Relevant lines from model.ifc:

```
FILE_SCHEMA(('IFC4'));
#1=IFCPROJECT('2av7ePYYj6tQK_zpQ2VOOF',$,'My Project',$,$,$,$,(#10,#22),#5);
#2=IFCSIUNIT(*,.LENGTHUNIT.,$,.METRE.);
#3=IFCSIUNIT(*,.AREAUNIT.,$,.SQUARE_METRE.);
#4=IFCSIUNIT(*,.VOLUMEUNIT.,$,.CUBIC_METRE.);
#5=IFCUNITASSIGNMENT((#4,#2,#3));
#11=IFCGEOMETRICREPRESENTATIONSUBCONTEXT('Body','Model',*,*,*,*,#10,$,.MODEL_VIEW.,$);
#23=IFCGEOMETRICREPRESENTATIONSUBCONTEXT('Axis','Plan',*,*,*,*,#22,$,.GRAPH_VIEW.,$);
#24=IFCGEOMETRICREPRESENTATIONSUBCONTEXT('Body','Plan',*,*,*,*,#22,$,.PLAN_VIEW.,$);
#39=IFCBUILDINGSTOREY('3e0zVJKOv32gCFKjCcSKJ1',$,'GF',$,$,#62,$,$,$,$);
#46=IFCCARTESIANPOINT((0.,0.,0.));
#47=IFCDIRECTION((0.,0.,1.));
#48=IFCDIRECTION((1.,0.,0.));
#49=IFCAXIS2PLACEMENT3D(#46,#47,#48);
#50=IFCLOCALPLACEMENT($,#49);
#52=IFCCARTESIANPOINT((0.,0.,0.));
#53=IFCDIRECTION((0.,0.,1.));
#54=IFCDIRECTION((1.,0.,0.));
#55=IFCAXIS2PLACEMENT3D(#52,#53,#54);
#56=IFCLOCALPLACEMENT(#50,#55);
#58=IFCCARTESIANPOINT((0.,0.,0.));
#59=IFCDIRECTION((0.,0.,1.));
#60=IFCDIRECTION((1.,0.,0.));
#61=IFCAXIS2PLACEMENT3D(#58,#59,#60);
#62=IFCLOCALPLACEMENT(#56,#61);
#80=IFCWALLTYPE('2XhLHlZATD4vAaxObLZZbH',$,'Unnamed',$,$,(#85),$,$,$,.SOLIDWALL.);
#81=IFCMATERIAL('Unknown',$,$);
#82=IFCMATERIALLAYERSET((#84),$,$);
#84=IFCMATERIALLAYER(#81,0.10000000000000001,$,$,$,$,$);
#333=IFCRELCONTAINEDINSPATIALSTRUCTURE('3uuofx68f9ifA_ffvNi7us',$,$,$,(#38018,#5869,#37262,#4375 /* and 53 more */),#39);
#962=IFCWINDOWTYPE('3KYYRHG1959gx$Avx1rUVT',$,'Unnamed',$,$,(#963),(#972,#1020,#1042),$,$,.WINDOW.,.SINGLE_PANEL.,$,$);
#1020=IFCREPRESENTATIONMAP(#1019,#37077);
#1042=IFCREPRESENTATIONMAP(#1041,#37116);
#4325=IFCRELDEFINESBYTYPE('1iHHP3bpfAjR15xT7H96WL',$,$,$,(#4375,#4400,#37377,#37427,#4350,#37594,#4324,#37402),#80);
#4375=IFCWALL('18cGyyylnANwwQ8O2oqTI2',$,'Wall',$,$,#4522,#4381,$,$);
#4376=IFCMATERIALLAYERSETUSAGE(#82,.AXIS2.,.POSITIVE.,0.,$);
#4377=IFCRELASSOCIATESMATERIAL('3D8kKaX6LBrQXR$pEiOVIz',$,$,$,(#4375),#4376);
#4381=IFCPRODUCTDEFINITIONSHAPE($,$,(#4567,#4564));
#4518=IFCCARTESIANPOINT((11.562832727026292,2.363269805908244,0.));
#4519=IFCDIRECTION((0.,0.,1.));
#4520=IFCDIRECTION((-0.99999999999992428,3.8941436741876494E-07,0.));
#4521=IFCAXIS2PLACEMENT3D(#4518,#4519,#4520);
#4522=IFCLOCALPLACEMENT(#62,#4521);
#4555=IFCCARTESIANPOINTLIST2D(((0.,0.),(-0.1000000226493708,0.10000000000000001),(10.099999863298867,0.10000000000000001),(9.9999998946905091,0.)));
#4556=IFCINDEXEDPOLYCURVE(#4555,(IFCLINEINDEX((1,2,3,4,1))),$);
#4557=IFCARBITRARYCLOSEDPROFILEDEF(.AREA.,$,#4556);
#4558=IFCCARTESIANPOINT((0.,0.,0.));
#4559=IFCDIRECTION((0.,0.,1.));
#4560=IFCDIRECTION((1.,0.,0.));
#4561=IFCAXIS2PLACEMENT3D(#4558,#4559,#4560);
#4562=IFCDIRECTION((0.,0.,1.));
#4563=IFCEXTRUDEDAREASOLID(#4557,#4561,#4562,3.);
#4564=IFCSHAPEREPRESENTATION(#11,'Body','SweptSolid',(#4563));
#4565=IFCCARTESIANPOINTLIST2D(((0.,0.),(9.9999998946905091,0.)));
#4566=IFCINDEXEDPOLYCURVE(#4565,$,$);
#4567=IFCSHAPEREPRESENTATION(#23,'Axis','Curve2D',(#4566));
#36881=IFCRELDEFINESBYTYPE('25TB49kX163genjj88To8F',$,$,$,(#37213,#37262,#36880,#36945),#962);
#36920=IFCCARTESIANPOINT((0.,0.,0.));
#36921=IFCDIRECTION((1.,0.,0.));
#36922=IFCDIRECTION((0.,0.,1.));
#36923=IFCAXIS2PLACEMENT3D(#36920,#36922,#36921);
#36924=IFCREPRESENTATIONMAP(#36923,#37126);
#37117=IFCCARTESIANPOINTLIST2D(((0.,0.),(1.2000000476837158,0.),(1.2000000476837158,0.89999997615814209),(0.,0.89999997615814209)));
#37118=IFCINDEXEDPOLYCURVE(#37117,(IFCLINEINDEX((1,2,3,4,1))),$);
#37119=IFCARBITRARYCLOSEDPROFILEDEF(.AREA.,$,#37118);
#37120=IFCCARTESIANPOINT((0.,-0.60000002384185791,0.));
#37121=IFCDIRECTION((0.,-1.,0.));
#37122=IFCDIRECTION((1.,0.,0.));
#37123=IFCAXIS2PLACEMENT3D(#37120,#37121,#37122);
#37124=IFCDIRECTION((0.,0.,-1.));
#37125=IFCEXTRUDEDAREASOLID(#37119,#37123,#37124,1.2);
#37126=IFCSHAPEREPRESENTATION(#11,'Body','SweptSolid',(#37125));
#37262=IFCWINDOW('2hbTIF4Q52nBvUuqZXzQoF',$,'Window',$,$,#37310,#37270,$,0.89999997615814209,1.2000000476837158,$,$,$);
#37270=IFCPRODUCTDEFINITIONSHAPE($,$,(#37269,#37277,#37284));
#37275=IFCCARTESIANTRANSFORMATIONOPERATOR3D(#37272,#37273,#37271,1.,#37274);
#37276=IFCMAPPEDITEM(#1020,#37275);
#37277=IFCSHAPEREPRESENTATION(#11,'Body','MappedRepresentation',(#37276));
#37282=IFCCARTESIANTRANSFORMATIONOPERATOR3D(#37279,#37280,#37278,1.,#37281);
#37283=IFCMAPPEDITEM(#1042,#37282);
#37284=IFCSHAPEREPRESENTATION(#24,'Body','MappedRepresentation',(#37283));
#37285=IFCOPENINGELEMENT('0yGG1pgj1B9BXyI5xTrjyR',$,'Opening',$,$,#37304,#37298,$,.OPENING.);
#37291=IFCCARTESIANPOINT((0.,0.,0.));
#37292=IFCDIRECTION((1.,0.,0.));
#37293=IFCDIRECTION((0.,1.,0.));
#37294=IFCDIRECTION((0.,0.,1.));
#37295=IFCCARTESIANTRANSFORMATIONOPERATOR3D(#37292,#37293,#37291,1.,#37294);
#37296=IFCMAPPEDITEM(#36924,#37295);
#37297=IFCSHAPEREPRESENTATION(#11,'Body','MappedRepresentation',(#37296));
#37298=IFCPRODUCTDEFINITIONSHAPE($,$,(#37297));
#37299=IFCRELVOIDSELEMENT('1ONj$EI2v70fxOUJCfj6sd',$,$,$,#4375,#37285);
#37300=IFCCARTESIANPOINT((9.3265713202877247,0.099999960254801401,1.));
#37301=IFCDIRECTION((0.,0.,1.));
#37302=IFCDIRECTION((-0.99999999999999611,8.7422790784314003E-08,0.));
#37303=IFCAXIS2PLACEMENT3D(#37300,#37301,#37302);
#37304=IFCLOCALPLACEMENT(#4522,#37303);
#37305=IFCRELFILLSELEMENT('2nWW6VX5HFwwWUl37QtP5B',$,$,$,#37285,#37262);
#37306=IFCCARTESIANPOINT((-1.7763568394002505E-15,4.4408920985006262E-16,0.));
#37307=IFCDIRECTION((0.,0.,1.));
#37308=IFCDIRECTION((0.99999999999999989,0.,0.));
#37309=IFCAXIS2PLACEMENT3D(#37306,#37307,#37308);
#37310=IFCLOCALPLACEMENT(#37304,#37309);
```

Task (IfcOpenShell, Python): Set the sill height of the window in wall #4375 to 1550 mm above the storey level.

```python
import numpy as np
import ifcopenshell
import ifcopenshell.api.geometry
import ifcopenshell.geom
import ifcopenshell.util.element
import ifcopenshell.util.placement
import ifcopenshell.util.shape
import ifcopenshell.util.unit

model = ifcopenshell.open("model.ifc")
unit_scale = ifcopenshell.util.unit.calculate_unit_scale(model)

window = model.by_guid("2hbTIF4Q52nBvUuqZXzQoF")
opening = window.FillsVoids[0].RelatingOpeningElement
storey = ifcopenshell.util.element.get_container(window, ifc_class="IfcBuildingStorey")
level = ifcopenshell.util.placement.get_local_placement(storey.ObjectPlacement)[2, 3]

# The opening's origin need not be at the sill, so measure its lowest point.
shape = ifcopenshell.geom.create_shape(ifcopenshell.geom.settings(), opening)
bottom = ifcopenshell.util.shape.get_shape_bottom_elevation(shape, shape.geometry) / unit_scale
dz = level + 1.55 / unit_scale - bottom

shift = np.array([0.0, 0.0, dz])
# The window is placed relative to its opening, so it follows when the opening moves.
matrix = ifcopenshell.util.placement.get_local_placement(opening.ObjectPlacement)
matrix[:3, 3] += shift
ifcopenshell.api.geometry.edit_object_placement(
    model, product=opening, matrix=matrix, is_si=False, should_transform_children=True
)

print(f"moved by {dz * unit_scale:+.3f} m")

model.write("model-out.ifc")
```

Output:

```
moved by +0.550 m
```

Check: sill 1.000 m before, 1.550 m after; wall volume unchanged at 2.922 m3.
